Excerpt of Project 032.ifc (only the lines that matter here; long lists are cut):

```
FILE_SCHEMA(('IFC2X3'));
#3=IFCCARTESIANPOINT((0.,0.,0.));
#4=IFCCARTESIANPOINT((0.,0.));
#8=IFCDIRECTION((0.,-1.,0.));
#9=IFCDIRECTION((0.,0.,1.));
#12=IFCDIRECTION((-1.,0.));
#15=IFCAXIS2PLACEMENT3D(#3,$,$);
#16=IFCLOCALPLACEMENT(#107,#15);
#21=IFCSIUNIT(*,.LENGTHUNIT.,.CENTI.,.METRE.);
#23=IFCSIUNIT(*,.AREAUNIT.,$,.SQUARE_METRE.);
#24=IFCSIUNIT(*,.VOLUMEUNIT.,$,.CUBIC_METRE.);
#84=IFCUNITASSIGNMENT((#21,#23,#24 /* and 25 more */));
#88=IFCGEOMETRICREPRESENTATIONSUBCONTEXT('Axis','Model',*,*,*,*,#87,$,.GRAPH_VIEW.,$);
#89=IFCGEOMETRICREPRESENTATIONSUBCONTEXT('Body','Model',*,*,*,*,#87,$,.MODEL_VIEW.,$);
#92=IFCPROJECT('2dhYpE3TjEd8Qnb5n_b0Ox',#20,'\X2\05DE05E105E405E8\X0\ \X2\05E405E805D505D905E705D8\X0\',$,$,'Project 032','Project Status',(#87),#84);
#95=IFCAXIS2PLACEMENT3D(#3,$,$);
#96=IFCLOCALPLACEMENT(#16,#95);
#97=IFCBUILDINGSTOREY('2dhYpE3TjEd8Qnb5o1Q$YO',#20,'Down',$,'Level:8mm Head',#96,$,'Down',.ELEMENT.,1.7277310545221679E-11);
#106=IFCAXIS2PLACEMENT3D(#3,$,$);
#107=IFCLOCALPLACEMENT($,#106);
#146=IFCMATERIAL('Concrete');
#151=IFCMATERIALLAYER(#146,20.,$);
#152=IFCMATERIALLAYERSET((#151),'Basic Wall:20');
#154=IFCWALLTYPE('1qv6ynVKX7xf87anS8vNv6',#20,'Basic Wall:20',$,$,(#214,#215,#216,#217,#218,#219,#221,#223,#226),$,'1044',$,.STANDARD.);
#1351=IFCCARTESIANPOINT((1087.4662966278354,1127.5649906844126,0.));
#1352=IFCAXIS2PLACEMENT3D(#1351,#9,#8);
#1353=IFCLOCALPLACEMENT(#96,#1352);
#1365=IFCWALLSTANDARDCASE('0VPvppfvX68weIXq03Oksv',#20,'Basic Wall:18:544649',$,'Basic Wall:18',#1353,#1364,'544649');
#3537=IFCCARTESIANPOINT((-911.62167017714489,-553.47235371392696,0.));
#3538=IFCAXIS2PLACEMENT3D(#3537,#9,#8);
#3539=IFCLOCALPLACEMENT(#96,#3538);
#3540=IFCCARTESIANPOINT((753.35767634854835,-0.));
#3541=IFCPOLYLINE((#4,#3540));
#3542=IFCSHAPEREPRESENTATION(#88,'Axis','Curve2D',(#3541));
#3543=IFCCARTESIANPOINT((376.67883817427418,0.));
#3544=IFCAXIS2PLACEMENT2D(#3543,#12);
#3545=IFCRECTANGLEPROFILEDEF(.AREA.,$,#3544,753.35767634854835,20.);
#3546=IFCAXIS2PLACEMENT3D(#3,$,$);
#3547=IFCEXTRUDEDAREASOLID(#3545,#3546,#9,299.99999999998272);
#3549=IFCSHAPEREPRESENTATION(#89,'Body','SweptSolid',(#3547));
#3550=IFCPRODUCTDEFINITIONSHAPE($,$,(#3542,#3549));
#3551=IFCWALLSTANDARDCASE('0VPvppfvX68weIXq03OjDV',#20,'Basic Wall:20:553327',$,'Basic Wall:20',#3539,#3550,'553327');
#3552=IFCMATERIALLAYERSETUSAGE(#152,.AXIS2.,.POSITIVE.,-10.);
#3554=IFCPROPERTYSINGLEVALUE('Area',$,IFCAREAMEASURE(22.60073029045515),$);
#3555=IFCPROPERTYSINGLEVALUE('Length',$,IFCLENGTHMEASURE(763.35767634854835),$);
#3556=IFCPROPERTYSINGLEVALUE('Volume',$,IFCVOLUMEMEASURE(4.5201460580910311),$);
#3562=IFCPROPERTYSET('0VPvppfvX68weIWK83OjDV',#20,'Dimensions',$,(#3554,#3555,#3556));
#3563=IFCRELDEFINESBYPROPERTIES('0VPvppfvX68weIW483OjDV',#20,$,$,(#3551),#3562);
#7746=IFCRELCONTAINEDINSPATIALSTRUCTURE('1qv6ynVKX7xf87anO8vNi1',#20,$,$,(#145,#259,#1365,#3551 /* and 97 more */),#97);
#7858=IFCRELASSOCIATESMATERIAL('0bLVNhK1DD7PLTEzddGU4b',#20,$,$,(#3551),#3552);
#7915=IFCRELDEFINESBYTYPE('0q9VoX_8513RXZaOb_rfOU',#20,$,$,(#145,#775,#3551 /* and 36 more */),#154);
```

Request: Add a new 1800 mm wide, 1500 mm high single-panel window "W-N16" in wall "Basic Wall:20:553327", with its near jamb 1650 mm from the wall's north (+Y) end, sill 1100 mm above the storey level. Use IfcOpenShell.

```python
import numpy as np
import ifcopenshell
import ifcopenshell.api.feature
import ifcopenshell.api.geometry
import ifcopenshell.api.pset
import ifcopenshell.api.root
import ifcopenshell.api.spatial
import ifcopenshell.api.type
import ifcopenshell.geom
import ifcopenshell.util.element
import ifcopenshell.util.placement
import ifcopenshell.util.representation
import ifcopenshell.util.shape
import ifcopenshell.util.unit

model = ifcopenshell.open("Project 032.ifc")
unit_scale = ifcopenshell.util.unit.calculate_unit_scale(model)
area_scale = ifcopenshell.util.unit.calculate_unit_scale(model, "AREAUNIT")
volume_scale = ifcopenshell.util.unit.calculate_unit_scale(model, "VOLUMEUNIT")
settings = ifcopenshell.geom.settings()


def volume(element):
    """Net volume in cubic metres, openings subtracted."""
    shape = ifcopenshell.geom.create_shape(settings, element)
    return ifcopenshell.util.shape.get_volume(shape.geometry)


wall = model.by_id(3551)
storey = ifcopenshell.util.element.get_container(wall, ifc_class="IfcBuildingStorey")
context = ifcopenshell.util.representation.get_context(model, "Model", "Body", "MODEL_VIEW")
before = volume(wall)

width, height, from_end, sill = 1.8, 1.5, 1.65, 1.1  # metres

# The wall runs along its own X axis, and the end named is its -X end.
wall_shape = ifcopenshell.geom.create_shape(settings, wall)
x, y, z = ifcopenshell.util.shape.get_vertices(wall_shape.geometry).T
start = x.min() + from_end
face, thickness = float(y.min()), float(y.max() - y.min())
wall_matrix = ifcopenshell.util.placement.get_local_placement(wall.ObjectPlacement)
level = ifcopenshell.util.placement.get_local_placement(storey.ObjectPlacement)[2, 3]


def in_wall(x, y):
    """Placement at x, y metres in the wall's axes, at sill height."""
    matrix = wall_matrix.copy()
    matrix[:, 3] = wall_matrix @ np.array([x / unit_scale, y / unit_scale, 0.0, 1.0])
    matrix[2, 3] = level + sill / unit_scale
    return matrix


# Opening: a box that overshoots both wall faces by 50 mm.
opening = ifcopenshell.api.root.create_entity(model, ifc_class="IfcOpeningElement")
box = ifcopenshell.api.geometry.add_wall_representation(
    model, context=context, length=width, height=height, thickness=thickness + 0.1
)
ifcopenshell.api.geometry.assign_representation(model, product=opening, representation=box)
ifcopenshell.api.geometry.edit_object_placement(model, product=opening, matrix=in_wall(start, face - 0.05), is_si=False)
ifcopenshell.api.feature.add_feature(model, feature=opening, element=wall)

window = ifcopenshell.api.root.create_entity(model, ifc_class="IfcWindow", name="W-N16")
window.OverallWidth, window.OverallHeight = width / unit_scale, height / unit_scale
body = ifcopenshell.api.geometry.add_window_representation(
    model,
    context=context,
    overall_width=window.OverallWidth,
    overall_height=window.OverallHeight,
    partition_type="SINGLE_PANEL",
)
ifcopenshell.api.geometry.assign_representation(model, product=window, representation=body)
ifcopenshell.api.spatial.assign_container(model, products=[window], relating_structure=storey)
fills = ifcopenshell.api.feature.add_filling(model, opening=opening, element=window)
fills.OwnerHistory = window.OwnerHistory  # required in IFC2X3

# IFC2X3 keeps the operation on the window style.
style = ifcopenshell.api.root.create_entity(model, ifc_class="IfcWindowStyle", name="W-N16")
style.OperationType, style.ConstructionType = "SINGLE_PANEL", "NOTDEFINED"
style.ParameterTakesPrecedence = style.Sizeable = False
ifcopenshell.api.type.assign_type(model, related_objects=[window], relating_type=style)

# Centre the window in the wall's thickness.
ifcopenshell.api.geometry.edit_object_placement(model, product=window, matrix=in_wall(start, face), is_si=False)
window_shape = ifcopenshell.geom.create_shape(settings, window)
depth = ifcopenshell.util.shape.get_vertices(window_shape.geometry)[:, 1]
offset = face + thickness / 2 - (depth.min() + depth.max()) / 2
ifcopenshell.api.geometry.edit_object_placement(model, product=window, matrix=in_wall(start, offset), is_si=False)

after = volume(wall)

# Update the wall's stored quantities.
pset = model.by_id(ifcopenshell.util.element.get_pset(wall, "Dimensions", should_inherit=False)["id"])
ifcopenshell.api.pset.edit_pset(model, pset=pset, properties={
    "Area": model.create_entity("IfcAreaMeasure", after / thickness / area_scale),
    "Volume": model.create_entity("IfcVolumeMeasure", after / volume_scale),
})

print(f"wall volume {before:.3f} -> {after:.3f} m3")

model.write("Project 032_v2.ifc")
```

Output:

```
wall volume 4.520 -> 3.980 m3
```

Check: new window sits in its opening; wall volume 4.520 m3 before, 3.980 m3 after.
